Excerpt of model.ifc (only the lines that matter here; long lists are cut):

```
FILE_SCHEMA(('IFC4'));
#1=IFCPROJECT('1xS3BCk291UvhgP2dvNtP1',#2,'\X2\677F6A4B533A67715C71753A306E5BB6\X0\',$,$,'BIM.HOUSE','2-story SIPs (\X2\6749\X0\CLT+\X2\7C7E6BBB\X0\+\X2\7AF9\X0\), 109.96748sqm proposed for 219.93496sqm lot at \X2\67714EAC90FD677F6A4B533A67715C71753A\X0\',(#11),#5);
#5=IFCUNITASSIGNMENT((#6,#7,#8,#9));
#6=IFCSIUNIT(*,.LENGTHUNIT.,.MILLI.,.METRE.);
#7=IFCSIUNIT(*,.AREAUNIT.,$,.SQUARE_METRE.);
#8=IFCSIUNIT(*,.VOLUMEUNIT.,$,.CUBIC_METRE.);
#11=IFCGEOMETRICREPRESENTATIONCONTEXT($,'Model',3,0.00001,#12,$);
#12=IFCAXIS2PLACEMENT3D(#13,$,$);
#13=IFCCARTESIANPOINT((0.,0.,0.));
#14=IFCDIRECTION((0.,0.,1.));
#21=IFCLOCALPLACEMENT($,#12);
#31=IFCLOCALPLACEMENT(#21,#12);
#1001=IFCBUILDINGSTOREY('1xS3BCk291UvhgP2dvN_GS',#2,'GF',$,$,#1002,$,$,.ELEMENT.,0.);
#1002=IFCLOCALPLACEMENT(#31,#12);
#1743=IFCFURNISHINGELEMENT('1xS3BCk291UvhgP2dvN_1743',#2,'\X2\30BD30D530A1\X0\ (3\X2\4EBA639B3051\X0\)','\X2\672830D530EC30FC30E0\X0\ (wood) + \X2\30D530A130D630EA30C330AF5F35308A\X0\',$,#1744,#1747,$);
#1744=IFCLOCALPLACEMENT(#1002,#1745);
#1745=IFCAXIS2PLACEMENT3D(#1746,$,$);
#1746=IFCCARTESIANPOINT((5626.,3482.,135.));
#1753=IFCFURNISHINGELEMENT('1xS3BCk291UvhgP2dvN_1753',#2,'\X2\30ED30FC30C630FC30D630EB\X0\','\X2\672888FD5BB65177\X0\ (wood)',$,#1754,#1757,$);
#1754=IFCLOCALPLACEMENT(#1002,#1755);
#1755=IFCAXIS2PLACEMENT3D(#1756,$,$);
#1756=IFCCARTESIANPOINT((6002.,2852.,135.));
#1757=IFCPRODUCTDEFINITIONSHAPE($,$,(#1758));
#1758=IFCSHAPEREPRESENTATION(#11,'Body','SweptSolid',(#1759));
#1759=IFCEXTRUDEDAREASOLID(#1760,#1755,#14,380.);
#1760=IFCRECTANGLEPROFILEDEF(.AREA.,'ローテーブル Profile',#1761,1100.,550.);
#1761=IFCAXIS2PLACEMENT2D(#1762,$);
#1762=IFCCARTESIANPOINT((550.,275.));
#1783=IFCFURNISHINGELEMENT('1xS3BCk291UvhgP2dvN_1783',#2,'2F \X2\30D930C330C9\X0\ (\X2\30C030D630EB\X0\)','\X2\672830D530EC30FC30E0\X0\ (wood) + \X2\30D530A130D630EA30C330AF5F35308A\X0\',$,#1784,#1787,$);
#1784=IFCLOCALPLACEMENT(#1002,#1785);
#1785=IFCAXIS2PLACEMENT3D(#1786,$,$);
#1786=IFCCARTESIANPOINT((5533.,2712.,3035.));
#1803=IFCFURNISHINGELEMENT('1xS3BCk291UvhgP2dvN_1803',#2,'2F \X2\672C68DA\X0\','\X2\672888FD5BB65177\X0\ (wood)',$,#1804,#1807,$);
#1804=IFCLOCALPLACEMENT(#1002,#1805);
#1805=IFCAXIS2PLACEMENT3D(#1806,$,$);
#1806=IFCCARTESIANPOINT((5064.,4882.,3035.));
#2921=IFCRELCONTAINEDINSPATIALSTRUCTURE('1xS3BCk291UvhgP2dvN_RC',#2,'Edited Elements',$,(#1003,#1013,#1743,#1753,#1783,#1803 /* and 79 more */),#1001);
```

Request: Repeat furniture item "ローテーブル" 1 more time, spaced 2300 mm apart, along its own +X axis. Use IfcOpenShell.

```python
import ifcopenshell
import ifcopenshell.api.geometry
import ifcopenshell.api.root
import ifcopenshell.util.element
import ifcopenshell.util.placement

model = ifcopenshell.open("model.ifc")


def reuse_history(source, copy):
    """copy_class also copies each property set's owner history, people and application; keep the originals."""
    for rel in copy.IsDefinedBy:
        if rel.is_a("IfcRelDefinesByProperties") and (history := rel.RelatingPropertyDefinition.OwnerHistory):
            rel.RelatingPropertyDefinition.OwnerHistory = source.OwnerHistory
            ifcopenshell.util.element.remove_deep2(model, history)


source = model.by_guid("1xS3BCk291UvhgP2dvN_1753")
base = ifcopenshell.util.placement.get_local_placement(source.ObjectPlacement)
step = base[:3, 0] * 2300.0

for i in range(1, 2):
    copy = ifcopenshell.api.root.copy_class(model, product=source)
    copy.Representation = ifcopenshell.util.element.copy_deep(
        model, source.Representation, exclude=["IfcGeometricRepresentationContext", "IfcRepresentationMap"]
    )
    reuse_history(source, copy)
    matrix = base.copy()
    matrix[:3, 3] += i * step
    print("added at", matrix[:3, 3].round(3) + 0.0)
    ifcopenshell.api.geometry.edit_object_placement(model, product=copy, matrix=matrix, is_si=False)

model.write("model_v2.ifc")
```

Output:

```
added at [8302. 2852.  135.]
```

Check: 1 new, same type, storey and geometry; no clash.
